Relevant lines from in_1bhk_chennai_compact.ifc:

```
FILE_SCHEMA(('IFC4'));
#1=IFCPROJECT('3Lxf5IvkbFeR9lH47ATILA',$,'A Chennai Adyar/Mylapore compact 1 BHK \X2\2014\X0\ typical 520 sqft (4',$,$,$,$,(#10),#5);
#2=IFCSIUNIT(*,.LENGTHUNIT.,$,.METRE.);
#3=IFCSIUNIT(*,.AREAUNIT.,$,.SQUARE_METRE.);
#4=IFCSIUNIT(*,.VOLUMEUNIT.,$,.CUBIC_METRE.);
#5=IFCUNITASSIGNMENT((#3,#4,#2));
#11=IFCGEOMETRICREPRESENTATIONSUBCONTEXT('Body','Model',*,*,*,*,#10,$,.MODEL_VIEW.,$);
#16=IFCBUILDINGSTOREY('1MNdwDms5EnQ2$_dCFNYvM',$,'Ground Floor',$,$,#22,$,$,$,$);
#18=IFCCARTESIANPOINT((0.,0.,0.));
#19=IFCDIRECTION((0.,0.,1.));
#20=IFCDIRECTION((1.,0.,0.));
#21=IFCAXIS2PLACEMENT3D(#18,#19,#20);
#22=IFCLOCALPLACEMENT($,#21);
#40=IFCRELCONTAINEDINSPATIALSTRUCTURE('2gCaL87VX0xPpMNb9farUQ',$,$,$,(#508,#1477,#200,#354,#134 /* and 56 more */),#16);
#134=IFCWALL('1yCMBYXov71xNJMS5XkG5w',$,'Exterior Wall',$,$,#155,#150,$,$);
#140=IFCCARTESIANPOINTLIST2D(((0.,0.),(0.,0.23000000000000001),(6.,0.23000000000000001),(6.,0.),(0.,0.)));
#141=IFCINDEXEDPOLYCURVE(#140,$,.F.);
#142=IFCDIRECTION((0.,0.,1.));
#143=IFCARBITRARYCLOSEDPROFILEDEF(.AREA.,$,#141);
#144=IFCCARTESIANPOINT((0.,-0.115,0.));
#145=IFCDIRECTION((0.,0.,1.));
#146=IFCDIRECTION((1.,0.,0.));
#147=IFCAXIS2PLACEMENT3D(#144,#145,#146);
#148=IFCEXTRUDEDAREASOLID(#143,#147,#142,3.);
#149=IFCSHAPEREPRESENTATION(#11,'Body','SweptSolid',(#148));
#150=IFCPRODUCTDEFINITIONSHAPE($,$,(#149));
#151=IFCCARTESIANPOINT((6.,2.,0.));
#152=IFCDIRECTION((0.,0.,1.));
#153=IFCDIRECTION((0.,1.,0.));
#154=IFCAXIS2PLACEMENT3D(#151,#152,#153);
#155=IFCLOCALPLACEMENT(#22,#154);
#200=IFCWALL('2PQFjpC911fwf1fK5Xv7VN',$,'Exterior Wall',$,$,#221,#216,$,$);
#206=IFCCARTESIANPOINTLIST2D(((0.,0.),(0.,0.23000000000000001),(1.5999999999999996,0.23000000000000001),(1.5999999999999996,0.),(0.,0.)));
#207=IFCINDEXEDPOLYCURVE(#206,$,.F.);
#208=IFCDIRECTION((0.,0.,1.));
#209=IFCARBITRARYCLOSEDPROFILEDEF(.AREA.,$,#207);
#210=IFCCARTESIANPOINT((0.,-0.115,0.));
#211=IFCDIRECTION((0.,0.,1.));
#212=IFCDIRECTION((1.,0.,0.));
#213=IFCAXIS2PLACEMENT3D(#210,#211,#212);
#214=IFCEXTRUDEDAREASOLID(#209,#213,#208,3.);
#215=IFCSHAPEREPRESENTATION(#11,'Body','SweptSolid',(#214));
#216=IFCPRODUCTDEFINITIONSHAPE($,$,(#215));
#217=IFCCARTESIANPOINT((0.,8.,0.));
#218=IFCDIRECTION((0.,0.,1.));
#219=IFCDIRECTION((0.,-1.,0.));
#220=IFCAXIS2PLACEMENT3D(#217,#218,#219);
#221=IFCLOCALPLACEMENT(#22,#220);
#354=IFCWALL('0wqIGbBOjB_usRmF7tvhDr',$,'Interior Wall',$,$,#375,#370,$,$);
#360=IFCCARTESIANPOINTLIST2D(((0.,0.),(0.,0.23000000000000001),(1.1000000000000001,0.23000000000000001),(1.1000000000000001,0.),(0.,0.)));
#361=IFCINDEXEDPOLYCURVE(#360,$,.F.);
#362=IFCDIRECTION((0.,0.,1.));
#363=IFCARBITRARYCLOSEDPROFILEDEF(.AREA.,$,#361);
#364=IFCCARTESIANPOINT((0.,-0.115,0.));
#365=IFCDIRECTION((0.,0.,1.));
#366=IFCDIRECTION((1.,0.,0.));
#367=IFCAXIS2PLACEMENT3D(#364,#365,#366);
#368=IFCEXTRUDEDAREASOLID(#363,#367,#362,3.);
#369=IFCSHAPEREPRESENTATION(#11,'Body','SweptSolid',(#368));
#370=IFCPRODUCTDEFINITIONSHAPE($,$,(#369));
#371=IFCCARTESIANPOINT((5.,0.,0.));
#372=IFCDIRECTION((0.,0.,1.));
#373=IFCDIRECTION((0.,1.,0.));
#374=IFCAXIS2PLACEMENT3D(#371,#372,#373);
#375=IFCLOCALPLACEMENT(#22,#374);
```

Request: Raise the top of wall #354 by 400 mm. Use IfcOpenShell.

```python
import ifcopenshell
import ifcopenshell.geom
import ifcopenshell.util.representation
import ifcopenshell.util.shape

model = ifcopenshell.open("in_1bhk_chennai_compact.ifc")
settings = ifcopenshell.geom.settings()


def volume(element):
    """Net volume in cubic metres, openings subtracted."""
    shape = ifcopenshell.geom.create_shape(settings, element)
    return ifcopenshell.util.shape.get_volume(shape.geometry)


wall = model.by_guid("0wqIGbBOjB_usRmF7tvhDr")
before = volume(wall)

body = ifcopenshell.util.representation.get_representation(wall, "Model", "Body")
solid = body.Items[0]
old_height = solid.Depth
solid.Depth += 0.4
after = volume(wall)

print(f"height {old_height:g} -> {solid.Depth:g}, volume {before:.3f} -> {after:.3f} m3")

model.write("in_1bhk_chennai_compact-out.ifc")
```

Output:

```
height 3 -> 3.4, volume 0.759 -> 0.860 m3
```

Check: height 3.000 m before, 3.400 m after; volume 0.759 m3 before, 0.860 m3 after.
